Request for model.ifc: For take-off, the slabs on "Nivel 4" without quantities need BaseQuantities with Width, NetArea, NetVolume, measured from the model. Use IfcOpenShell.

First a look at what the model holds.

```python
import ifcopenshell
import ifcopenshell.util.element
import ifcopenshell.util.unit

model = ifcopenshell.open("model.ifc")
print(model.schema)
for unit_type in ("LENGTHUNIT", "AREAUNIT", "VOLUMEUNIT"):
    print(unit_type, ifcopenshell.util.unit.calculate_unit_scale(model, unit_type))
storey = next(s for s in model.by_type("IfcBuildingStorey") if s.Name == "Nivel 4")
slabs = [e for e in ifcopenshell.util.element.get_decomposition(storey) if e.is_a("IfcSlab")]
for e in sorted(slabs, key=lambda e: e.id()):
    print(e.id(), e.is_a(), e.Name, list(ifcopenshell.util.element.get_psets(e, qtos_only=True)), sep=" | ")
```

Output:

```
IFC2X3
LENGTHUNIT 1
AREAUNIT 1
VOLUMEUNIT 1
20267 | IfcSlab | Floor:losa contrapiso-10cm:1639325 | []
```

```python
import ifcopenshell
import ifcopenshell.api.pset
import ifcopenshell.geom
import ifcopenshell.util.element
import ifcopenshell.util.shape
import ifcopenshell.util.unit

model = ifcopenshell.open("model.ifc")
unit_scale = ifcopenshell.util.unit.calculate_unit_scale(model)
area_scale = ifcopenshell.util.unit.calculate_unit_scale(model, "AREAUNIT")
volume_scale = ifcopenshell.util.unit.calculate_unit_scale(model, "VOLUMEUNIT")
settings = ifcopenshell.geom.settings()

storey = next(s for s in model.by_type("IfcBuildingStorey") if s.Name == "Nivel 4")
slabs = [e for e in ifcopenshell.util.element.get_decomposition(storey) if e.is_a("IfcSlab")]

for e in sorted(slabs, key=lambda e: e.id()):
    if ifcopenshell.util.element.get_psets(e, qtos_only=True, should_inherit=False):
        continue
    # Geometry comes back in metres, in the element's own axes.
    shape = ifcopenshell.geom.create_shape(settings, e)
    values = {
        "Width": ifcopenshell.util.shape.get_z(shape.geometry) / unit_scale,
        "NetArea": ifcopenshell.util.shape.get_footprint_area(shape.geometry) / area_scale,
        "NetVolume": ifcopenshell.util.shape.get_volume(shape.geometry) / volume_scale,
    }
    qto = ifcopenshell.api.pset.add_qto(model, product=e, name="BaseQuantities")
    ifcopenshell.api.pset.edit_qto(model, qto=qto, properties=values)
    print(e.id(), {k: round(v, 3) for k, v in values.items()})

model.write("model_rev.ifc")
```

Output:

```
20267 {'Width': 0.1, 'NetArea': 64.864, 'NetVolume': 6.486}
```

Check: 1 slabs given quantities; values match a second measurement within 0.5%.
